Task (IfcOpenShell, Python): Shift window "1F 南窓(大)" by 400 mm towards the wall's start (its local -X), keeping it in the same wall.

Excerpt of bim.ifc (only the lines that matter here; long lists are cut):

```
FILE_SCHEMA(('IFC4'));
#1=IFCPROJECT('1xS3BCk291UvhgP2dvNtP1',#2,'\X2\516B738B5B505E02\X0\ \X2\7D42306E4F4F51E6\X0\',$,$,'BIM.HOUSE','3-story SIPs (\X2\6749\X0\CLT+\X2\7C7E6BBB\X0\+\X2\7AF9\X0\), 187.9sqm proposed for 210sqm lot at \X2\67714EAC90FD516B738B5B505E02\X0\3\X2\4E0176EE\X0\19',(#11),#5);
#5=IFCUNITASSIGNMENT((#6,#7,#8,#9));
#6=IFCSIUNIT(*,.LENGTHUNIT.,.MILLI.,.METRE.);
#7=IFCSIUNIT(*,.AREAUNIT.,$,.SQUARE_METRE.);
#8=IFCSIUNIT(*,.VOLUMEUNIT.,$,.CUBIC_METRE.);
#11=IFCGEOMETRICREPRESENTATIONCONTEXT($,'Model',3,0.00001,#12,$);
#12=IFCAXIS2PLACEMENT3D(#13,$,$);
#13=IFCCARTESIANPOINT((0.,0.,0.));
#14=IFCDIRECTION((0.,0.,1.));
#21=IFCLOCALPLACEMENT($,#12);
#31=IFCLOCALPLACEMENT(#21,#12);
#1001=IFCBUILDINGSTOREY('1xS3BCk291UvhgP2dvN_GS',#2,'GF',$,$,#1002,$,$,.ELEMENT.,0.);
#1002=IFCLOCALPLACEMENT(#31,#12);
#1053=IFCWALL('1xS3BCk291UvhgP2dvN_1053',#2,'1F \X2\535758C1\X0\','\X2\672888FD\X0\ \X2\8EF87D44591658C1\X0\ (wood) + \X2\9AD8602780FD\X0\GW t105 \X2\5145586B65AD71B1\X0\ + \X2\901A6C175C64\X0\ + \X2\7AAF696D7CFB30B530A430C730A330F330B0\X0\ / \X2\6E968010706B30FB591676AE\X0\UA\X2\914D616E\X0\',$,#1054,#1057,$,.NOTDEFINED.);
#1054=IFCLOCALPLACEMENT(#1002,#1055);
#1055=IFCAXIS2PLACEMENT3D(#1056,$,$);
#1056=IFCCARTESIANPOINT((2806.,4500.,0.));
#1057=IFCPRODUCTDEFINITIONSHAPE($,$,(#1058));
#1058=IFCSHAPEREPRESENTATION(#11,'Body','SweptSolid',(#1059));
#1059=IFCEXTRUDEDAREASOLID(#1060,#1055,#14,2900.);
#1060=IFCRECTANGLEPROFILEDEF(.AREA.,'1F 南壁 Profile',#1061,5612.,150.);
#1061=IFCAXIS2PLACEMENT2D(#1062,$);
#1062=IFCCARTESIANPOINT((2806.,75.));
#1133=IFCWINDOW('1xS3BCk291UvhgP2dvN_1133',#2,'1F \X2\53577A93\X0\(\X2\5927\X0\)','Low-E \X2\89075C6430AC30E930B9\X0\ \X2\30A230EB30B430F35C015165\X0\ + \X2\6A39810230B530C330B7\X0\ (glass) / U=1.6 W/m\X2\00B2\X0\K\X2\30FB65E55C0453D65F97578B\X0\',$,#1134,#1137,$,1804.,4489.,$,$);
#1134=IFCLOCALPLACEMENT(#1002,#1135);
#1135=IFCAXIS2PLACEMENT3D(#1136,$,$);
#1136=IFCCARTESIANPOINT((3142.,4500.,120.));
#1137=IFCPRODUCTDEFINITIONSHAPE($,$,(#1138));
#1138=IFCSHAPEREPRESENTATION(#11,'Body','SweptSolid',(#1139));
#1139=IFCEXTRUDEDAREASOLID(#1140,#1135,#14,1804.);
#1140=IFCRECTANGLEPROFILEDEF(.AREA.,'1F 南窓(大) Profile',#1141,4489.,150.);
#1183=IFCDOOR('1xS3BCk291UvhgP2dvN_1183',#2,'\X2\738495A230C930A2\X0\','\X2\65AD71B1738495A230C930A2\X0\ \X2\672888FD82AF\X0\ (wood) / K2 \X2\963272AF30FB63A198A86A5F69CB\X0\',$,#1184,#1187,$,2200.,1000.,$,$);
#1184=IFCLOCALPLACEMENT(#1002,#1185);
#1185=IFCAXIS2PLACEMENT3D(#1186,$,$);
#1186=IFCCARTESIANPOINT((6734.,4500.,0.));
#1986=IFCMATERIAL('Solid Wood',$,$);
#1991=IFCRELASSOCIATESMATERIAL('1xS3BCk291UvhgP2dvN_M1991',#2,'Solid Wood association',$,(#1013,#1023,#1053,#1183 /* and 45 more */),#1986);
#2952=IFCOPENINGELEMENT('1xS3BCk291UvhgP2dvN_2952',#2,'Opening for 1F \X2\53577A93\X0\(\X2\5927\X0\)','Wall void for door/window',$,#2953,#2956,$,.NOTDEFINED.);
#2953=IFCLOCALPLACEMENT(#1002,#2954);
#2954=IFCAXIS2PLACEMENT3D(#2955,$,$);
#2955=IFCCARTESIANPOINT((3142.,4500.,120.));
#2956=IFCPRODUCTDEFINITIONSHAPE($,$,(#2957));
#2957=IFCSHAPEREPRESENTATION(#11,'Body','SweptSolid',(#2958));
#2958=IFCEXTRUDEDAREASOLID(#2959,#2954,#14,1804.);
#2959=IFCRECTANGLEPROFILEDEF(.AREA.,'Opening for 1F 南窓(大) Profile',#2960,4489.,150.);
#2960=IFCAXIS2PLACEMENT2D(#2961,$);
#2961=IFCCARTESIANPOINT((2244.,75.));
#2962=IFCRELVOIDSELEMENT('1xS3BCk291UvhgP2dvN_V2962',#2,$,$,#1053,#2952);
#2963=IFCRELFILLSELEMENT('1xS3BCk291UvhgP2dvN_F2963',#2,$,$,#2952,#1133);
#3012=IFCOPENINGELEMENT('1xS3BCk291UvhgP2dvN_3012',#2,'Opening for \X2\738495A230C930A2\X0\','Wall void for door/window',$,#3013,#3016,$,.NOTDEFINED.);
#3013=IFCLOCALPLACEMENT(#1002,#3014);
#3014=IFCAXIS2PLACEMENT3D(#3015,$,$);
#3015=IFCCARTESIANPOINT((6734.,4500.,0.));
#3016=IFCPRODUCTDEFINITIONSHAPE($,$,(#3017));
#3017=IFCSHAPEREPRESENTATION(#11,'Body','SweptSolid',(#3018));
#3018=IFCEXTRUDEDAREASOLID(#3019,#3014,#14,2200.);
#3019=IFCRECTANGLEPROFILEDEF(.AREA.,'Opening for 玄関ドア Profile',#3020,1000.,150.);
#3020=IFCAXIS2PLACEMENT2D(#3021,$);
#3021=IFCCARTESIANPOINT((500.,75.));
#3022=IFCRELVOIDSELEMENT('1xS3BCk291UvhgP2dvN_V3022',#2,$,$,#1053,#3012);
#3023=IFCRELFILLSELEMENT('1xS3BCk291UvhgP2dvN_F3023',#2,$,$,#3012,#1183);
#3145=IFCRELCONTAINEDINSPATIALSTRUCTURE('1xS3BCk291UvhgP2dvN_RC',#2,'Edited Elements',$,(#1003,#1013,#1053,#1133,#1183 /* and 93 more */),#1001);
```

```python
import ifcopenshell
import ifcopenshell.api.geometry
import ifcopenshell.util.placement
import ifcopenshell.util.unit

model = ifcopenshell.open("bim.ifc")
unit_scale = ifcopenshell.util.unit.calculate_unit_scale(model)

window = model.by_guid("1xS3BCk291UvhgP2dvN_1133")
opening = window.FillsVoids[0].RelatingOpeningElement
wall = opening.VoidsElements[0].RelatingBuildingElement

wall_matrix = ifcopenshell.util.placement.get_local_placement(wall.ObjectPlacement)
shift = wall_matrix[:3, 0] * -0.4 / unit_scale
before = ifcopenshell.util.placement.get_local_placement(window.ObjectPlacement)[:3, 3].copy()

# The window is not placed relative to its opening, so move both.
for product in (opening, window):
    matrix = ifcopenshell.util.placement.get_local_placement(product.ObjectPlacement)
    matrix[:3, 3] += shift
    ifcopenshell.api.geometry.edit_object_placement(model, product=product, matrix=matrix, is_si=False)

after = ifcopenshell.util.placement.get_local_placement(window.ObjectPlacement)[:3, 3]
print("window moved by", (after - before).round(3) + 0.0)

model.write("bim-out.ifc")
```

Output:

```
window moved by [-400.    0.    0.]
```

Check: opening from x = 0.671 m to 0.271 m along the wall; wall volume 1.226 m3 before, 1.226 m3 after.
